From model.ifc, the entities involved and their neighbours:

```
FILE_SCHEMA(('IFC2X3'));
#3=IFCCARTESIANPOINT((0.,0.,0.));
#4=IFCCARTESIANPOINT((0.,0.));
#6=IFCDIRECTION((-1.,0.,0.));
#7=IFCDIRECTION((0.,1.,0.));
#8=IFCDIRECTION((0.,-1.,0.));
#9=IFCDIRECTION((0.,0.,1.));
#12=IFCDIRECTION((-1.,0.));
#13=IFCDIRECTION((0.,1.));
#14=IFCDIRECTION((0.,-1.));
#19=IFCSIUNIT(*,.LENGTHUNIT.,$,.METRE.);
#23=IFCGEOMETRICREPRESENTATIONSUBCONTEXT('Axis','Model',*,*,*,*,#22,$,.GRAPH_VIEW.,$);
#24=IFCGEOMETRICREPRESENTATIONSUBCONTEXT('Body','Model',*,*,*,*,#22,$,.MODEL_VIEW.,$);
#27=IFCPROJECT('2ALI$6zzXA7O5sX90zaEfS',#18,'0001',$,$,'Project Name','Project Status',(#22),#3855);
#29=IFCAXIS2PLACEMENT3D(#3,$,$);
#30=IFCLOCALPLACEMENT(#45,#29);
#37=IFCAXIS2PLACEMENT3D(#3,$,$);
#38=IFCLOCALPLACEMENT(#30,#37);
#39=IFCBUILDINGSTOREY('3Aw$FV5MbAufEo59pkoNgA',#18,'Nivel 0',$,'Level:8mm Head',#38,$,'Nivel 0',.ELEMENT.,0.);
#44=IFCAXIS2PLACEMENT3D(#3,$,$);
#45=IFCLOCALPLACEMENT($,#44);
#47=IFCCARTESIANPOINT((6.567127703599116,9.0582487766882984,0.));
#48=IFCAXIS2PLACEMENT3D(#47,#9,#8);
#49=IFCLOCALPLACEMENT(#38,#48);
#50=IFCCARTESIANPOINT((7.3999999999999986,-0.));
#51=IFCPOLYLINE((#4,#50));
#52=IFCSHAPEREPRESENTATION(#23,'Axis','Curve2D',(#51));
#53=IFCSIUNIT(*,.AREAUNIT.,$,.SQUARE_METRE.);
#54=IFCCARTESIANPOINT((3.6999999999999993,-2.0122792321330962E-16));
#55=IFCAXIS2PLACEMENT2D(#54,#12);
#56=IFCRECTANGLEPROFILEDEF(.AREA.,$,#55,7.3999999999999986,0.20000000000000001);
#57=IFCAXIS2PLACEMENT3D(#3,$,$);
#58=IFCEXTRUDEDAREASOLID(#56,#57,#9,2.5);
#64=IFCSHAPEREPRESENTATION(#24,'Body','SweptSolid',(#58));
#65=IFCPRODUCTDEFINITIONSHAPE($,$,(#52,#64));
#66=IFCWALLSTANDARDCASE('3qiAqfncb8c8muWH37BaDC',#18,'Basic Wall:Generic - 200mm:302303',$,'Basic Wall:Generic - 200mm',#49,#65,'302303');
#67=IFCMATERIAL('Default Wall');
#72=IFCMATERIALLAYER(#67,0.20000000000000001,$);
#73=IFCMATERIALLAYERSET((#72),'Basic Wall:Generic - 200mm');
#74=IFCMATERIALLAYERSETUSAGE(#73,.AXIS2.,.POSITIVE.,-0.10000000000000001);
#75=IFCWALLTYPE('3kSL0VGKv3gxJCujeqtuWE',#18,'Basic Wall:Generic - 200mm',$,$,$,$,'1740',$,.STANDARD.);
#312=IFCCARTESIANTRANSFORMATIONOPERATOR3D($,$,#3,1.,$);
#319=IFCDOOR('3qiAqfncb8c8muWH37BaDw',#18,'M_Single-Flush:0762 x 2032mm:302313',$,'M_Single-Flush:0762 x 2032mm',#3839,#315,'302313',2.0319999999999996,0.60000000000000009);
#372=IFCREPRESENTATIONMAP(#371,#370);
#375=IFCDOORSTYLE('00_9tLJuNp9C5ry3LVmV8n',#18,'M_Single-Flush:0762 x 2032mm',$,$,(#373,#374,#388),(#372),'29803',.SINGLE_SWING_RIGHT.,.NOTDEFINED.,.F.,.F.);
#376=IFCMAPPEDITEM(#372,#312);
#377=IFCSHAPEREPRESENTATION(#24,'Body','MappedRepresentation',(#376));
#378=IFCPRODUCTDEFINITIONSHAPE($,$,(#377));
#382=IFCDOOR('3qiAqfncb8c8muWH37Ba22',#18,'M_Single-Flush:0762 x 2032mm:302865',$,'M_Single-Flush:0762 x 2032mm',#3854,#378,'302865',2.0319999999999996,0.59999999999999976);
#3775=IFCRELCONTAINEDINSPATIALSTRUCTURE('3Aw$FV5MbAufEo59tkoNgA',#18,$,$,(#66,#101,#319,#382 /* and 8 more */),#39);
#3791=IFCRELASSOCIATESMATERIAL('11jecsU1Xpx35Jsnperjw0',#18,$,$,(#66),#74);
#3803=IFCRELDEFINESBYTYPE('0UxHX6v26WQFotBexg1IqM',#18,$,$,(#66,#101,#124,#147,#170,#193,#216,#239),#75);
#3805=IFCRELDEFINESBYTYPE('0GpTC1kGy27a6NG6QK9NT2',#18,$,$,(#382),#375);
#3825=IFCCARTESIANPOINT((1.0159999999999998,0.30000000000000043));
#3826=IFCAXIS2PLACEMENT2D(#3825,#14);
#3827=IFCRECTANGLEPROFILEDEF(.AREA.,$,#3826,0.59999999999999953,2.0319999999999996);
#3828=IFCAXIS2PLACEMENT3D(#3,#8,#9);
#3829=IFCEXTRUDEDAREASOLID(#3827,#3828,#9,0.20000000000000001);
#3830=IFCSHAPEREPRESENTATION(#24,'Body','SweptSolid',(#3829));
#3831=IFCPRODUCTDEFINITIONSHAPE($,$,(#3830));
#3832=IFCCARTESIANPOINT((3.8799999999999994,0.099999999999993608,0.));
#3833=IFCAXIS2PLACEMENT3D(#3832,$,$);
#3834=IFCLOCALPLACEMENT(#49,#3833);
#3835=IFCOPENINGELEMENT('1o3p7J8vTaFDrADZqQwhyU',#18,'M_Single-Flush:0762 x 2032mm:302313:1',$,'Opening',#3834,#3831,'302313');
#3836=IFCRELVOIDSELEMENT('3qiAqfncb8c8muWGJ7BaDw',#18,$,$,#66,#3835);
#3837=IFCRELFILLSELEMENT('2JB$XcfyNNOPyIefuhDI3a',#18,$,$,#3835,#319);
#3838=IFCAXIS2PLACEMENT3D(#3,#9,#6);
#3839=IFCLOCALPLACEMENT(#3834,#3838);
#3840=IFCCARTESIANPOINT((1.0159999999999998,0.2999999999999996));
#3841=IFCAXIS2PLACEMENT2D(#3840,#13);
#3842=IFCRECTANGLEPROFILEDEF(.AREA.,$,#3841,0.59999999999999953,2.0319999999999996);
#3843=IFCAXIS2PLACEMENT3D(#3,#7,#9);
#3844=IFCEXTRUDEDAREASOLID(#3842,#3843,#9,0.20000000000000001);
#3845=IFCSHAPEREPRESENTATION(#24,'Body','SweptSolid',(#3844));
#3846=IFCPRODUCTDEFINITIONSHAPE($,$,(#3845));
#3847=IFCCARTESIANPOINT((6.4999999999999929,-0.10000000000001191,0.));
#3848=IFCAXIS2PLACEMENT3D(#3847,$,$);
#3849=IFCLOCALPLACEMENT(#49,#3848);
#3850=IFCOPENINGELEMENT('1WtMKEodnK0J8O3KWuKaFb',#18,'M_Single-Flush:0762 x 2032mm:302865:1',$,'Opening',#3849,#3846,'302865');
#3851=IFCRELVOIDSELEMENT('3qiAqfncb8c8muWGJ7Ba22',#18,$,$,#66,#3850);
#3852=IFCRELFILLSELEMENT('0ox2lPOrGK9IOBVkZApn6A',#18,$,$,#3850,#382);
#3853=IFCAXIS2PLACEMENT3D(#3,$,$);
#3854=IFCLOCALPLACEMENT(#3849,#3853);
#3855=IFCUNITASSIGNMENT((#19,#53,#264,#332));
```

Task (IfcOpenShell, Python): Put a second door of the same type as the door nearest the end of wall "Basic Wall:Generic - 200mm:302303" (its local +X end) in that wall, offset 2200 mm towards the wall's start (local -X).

```python
import ifcopenshell
import ifcopenshell.api.feature
import ifcopenshell.api.geometry
import ifcopenshell.api.root
import ifcopenshell.geom
import ifcopenshell.util.element
import ifcopenshell.util.placement
import ifcopenshell.util.shape

model = ifcopenshell.open("model.ifc")
settings = ifcopenshell.geom.settings()


def volume(element):
    """Net volume in cubic metres, openings subtracted."""
    shape = ifcopenshell.geom.create_shape(settings, element)
    return ifcopenshell.util.shape.get_volume(shape.geometry)


def reuse_history(source, copy):
    """copy_class also copies each property set's owner history, people and application; keep the originals."""
    for rel in copy.IsDefinedBy:
        if rel.is_a("IfcRelDefinesByProperties") and (history := rel.RelatingPropertyDefinition.OwnerHistory):
            rel.RelatingPropertyDefinition.OwnerHistory = source.OwnerHistory
            ifcopenshell.util.element.remove_deep2(model, history)


door = model.by_id(382)
opening = door.FillsVoids[0].RelatingOpeningElement
wall = opening.VoidsElements[0].RelatingBuildingElement
before = volume(wall)
shift = ifcopenshell.util.placement.get_local_placement(wall.ObjectPlacement)[:3, 0] * -2.2

# copy_class copies the void relationship, type, container and properties, but no geometry.
new_opening = ifcopenshell.api.root.copy_class(model, product=opening)
new_opening.Representation = ifcopenshell.util.element.copy_deep(
    model, opening.Representation, exclude=["IfcGeometricRepresentationContext", "IfcRepresentationMap"]
)
new_opening.Name = "M_Single-Flush:0762 x 2032mm"
new_opening.Tag = None
new_door = ifcopenshell.api.root.copy_class(model, product=door)
new_door.Representation = ifcopenshell.util.element.copy_deep(
    model, door.Representation, exclude=["IfcGeometricRepresentationContext", "IfcRepresentationMap"]
)
new_door.Name = "M_Single-Flush:0762 x 2032mm"
new_door.Tag = None
reuse_history(door, new_door)
fills = ifcopenshell.api.feature.add_filling(model, opening=new_opening, element=new_door)
fills.OwnerHistory = new_door.OwnerHistory  # required in IFC2X3

for old, new in ((opening, new_opening), (door, new_door)):
    matrix = ifcopenshell.util.placement.get_local_placement(old.ObjectPlacement)
    matrix[:3, 3] += shift
    ifcopenshell.api.geometry.edit_object_placement(model, product=new, matrix=matrix, is_si=False)

after = volume(wall)

print(f"wall volume {before:.3f} -> {after:.3f} m3")

model.write("model_edited.ifc")
```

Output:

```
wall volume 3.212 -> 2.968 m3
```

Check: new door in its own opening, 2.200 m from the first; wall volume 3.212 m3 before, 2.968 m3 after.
